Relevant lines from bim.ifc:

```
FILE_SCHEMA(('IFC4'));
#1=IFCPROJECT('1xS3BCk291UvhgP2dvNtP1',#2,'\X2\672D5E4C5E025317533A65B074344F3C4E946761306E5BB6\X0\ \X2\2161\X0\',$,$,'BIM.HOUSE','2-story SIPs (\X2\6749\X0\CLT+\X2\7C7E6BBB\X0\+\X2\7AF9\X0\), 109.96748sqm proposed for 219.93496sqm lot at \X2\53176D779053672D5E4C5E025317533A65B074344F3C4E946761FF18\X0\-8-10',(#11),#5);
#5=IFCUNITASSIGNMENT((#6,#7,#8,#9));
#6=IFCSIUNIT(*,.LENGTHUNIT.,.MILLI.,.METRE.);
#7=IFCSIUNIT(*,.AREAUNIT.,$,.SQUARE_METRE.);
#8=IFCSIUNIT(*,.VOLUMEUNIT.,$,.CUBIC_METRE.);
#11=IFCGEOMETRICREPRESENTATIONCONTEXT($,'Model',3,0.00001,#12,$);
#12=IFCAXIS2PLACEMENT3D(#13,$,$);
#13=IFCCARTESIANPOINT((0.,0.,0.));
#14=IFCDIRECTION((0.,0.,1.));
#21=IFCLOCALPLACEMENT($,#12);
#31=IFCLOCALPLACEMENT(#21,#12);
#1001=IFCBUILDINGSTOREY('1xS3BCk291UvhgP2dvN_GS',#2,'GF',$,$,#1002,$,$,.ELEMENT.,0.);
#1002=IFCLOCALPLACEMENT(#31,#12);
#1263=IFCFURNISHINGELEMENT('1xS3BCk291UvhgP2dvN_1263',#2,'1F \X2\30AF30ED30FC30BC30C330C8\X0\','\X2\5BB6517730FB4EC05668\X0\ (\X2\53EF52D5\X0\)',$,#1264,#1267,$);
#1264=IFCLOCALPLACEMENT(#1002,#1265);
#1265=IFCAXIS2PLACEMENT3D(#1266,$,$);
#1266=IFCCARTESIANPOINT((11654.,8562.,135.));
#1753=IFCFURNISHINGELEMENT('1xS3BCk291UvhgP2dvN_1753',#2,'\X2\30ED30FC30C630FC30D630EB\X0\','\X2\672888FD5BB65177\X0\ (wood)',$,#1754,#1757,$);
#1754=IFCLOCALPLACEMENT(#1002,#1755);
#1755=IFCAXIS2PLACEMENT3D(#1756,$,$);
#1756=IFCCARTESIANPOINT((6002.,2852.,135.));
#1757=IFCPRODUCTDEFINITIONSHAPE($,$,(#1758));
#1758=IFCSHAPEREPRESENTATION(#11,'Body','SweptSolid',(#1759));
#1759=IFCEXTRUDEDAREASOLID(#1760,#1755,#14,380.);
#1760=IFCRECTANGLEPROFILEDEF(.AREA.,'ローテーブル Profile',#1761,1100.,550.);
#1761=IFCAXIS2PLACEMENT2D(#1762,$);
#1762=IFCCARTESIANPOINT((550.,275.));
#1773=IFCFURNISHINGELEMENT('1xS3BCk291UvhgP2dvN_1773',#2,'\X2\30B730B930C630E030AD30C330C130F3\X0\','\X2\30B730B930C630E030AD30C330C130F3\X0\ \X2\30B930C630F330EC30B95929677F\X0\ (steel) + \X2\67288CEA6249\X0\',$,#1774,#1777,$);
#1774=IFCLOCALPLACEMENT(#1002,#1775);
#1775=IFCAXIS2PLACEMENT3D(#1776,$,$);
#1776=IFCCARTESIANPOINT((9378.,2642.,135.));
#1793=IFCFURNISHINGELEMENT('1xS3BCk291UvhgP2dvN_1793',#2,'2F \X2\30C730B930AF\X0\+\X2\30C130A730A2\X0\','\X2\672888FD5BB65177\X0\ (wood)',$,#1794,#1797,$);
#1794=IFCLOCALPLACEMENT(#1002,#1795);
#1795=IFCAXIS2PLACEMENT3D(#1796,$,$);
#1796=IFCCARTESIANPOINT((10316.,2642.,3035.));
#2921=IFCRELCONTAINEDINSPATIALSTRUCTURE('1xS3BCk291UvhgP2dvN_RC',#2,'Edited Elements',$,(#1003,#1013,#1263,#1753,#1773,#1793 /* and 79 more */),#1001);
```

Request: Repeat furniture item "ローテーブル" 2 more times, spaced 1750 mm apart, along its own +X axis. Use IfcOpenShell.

```python
import ifcopenshell
import ifcopenshell.api.geometry
import ifcopenshell.api.root
import ifcopenshell.util.element
import ifcopenshell.util.placement
import ifcopenshell.util.unit

model = ifcopenshell.open("bim.ifc")
unit_scale = ifcopenshell.util.unit.calculate_unit_scale(model)


def reuse_history(source, copy):
    """copy_class also copies each property set's owner history, people and application; keep the originals."""
    for rel in copy.IsDefinedBy:
        if rel.is_a("IfcRelDefinesByProperties") and (history := rel.RelatingPropertyDefinition.OwnerHistory):
            rel.RelatingPropertyDefinition.OwnerHistory = source.OwnerHistory
            ifcopenshell.util.element.remove_deep2(model, history)


source = model.by_id(1753)
base = ifcopenshell.util.placement.get_local_placement(source.ObjectPlacement)
step = base[:3, 0] * 1.75 / unit_scale

for i in range(1, 3):
    copy = ifcopenshell.api.root.copy_class(model, product=source)
    copy.Representation = ifcopenshell.util.element.copy_deep(
        model, source.Representation, exclude=["IfcGeometricRepresentationContext", "IfcRepresentationMap"]
    )
    reuse_history(source, copy)
    matrix = base.copy()
    matrix[:3, 3] += i * step
    print("added at", matrix[:3, 3].round(3) + 0.0)
    ifcopenshell.api.geometry.edit_object_placement(model, product=copy, matrix=matrix, is_si=False)

model.write("bim_edited.ifc")
```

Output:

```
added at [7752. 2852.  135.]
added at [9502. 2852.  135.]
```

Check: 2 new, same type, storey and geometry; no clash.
